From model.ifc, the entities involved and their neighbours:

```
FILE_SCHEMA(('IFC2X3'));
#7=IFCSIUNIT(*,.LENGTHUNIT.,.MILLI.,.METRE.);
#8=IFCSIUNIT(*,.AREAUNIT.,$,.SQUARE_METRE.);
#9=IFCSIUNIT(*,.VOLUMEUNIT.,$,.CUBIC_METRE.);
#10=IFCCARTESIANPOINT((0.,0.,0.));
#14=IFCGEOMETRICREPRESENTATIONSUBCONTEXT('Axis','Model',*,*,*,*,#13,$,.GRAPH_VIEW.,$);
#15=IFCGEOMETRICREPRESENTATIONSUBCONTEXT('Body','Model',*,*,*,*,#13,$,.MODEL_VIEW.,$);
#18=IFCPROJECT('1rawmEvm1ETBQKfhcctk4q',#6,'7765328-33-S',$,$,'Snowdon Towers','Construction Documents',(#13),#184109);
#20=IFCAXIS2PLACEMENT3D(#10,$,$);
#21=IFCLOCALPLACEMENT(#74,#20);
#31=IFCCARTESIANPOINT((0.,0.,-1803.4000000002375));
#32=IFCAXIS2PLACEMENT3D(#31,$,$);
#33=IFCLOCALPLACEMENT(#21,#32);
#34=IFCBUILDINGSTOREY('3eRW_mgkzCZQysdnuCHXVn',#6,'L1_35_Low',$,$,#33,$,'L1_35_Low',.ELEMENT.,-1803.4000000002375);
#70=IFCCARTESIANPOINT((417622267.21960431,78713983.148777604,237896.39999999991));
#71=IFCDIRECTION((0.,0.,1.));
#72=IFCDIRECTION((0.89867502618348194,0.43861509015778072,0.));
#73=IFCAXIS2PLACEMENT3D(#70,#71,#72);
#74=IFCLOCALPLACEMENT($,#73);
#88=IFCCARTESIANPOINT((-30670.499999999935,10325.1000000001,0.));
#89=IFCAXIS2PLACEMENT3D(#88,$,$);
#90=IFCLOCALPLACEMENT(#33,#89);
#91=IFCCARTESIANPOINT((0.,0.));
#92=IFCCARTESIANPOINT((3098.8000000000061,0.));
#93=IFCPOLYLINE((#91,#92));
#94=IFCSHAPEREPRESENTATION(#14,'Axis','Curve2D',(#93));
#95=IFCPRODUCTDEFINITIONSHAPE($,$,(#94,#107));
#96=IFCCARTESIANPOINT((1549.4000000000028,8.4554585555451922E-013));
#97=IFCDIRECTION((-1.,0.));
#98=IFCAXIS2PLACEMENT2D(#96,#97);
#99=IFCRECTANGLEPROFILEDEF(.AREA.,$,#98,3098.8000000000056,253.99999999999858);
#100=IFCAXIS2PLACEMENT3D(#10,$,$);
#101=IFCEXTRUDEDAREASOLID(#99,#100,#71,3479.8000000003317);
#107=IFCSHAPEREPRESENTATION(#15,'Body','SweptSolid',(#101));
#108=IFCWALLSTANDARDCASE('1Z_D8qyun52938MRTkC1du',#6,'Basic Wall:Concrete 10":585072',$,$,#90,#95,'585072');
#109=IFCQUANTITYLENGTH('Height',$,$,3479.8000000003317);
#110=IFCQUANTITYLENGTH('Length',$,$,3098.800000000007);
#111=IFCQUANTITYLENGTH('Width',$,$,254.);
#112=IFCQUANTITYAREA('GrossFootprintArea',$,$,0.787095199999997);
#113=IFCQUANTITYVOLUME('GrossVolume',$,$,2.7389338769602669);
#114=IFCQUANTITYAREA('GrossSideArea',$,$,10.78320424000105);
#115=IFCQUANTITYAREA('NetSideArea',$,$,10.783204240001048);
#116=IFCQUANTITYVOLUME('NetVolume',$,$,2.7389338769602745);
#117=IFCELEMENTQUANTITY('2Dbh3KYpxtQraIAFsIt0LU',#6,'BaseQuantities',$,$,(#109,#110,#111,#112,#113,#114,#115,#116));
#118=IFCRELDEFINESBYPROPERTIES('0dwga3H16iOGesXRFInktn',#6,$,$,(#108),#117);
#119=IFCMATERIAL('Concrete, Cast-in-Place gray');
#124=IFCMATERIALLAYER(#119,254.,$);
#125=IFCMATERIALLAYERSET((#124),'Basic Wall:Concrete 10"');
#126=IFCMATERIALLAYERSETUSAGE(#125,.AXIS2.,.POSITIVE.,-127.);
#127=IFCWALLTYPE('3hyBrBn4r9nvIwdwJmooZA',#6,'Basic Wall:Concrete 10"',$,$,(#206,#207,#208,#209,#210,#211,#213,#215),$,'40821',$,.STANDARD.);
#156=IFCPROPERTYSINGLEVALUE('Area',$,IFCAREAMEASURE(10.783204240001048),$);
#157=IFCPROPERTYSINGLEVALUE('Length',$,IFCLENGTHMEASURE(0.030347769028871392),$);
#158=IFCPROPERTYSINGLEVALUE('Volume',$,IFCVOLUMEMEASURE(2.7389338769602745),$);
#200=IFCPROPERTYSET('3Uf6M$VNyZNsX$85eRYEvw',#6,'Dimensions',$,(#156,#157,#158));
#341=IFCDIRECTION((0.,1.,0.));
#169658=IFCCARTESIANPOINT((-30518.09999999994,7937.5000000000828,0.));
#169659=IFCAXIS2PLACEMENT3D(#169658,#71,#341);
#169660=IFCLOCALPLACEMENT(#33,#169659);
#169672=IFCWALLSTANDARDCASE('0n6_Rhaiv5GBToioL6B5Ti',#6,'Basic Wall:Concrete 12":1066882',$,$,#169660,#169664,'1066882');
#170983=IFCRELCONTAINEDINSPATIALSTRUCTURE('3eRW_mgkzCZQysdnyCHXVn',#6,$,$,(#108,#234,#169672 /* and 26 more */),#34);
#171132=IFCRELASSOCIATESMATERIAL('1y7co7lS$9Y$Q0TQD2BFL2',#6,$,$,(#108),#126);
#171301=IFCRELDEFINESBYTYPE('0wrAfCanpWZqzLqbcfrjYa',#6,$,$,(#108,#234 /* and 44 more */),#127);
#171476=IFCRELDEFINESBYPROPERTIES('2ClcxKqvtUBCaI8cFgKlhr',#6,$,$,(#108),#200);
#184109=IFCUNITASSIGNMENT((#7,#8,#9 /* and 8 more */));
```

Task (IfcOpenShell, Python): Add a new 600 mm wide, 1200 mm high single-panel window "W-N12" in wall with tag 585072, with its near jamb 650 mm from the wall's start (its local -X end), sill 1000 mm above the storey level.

```python
import numpy as np
import ifcopenshell
import ifcopenshell.api.feature
import ifcopenshell.api.geometry
import ifcopenshell.api.pset
import ifcopenshell.api.root
import ifcopenshell.api.spatial
import ifcopenshell.api.type
import ifcopenshell.geom
import ifcopenshell.util.element
import ifcopenshell.util.placement
import ifcopenshell.util.representation
import ifcopenshell.util.shape
import ifcopenshell.util.unit

model = ifcopenshell.open("model.ifc")
unit_scale = ifcopenshell.util.unit.calculate_unit_scale(model)
area_scale = ifcopenshell.util.unit.calculate_unit_scale(model, "AREAUNIT")
volume_scale = ifcopenshell.util.unit.calculate_unit_scale(model, "VOLUMEUNIT")
settings = ifcopenshell.geom.settings()


def volume(element):
    """Net volume in cubic metres, openings subtracted."""
    shape = ifcopenshell.geom.create_shape(settings, element)
    return ifcopenshell.util.shape.get_volume(shape.geometry)


wall = model.by_guid("1Z_D8qyun52938MRTkC1du")
storey = ifcopenshell.util.element.get_container(wall, ifc_class="IfcBuildingStorey")
context = ifcopenshell.util.representation.get_context(model, "Model", "Body", "MODEL_VIEW")
before = volume(wall)

width, height, from_end, sill = 0.6, 1.2, 0.65, 1  # metres

# The wall runs along its own X axis, and the end named is its -X end.
wall_shape = ifcopenshell.geom.create_shape(settings, wall)
x, y, z = ifcopenshell.util.shape.get_vertices(wall_shape.geometry).T
start = x.min() + from_end
face, thickness = float(y.min()), float(y.max() - y.min())
wall_matrix = ifcopenshell.util.placement.get_local_placement(wall.ObjectPlacement)
level = ifcopenshell.util.placement.get_local_placement(storey.ObjectPlacement)[2, 3]


def in_wall(x, y):
    """Placement at x, y metres in the wall's axes, at sill height."""
    matrix = wall_matrix.copy()
    matrix[:, 3] = wall_matrix @ np.array([x / unit_scale, y / unit_scale, 0.0, 1.0])
    matrix[2, 3] = level + sill / unit_scale
    return matrix


# Opening: a box that overshoots both wall faces by 50 mm.
opening = ifcopenshell.api.root.create_entity(model, ifc_class="IfcOpeningElement")
box = ifcopenshell.api.geometry.add_wall_representation(
    model, context=context, length=width, height=height, thickness=thickness + 0.1
)
ifcopenshell.api.geometry.assign_representation(model, product=opening, representation=box)
ifcopenshell.api.geometry.edit_object_placement(model, product=opening, matrix=in_wall(start, face - 0.05), is_si=False)
ifcopenshell.api.feature.add_feature(model, feature=opening, element=wall)

window = ifcopenshell.api.root.create_entity(model, ifc_class="IfcWindow", name="W-N12")
window.OverallWidth, window.OverallHeight = width / unit_scale, height / unit_scale
body = ifcopenshell.api.geometry.add_window_representation(
    model,
    context=context,
    overall_width=window.OverallWidth,
    overall_height=window.OverallHeight,
    partition_type="SINGLE_PANEL",
)
ifcopenshell.api.geometry.assign_representation(model, product=window, representation=body)
ifcopenshell.api.spatial.assign_container(model, products=[window], relating_structure=storey)
fills = ifcopenshell.api.feature.add_filling(model, opening=opening, element=window)
fills.OwnerHistory = window.OwnerHistory  # required in IFC2X3

# IFC2X3 keeps the operation on the window style.
style = ifcopenshell.api.root.create_entity(model, ifc_class="IfcWindowStyle", name="W-N12")
style.OperationType, style.ConstructionType = "SINGLE_PANEL", "NOTDEFINED"
style.ParameterTakesPrecedence = style.Sizeable = False
ifcopenshell.api.type.assign_type(model, related_objects=[window], relating_type=style)

# Centre the window in the wall's thickness.
ifcopenshell.api.geometry.edit_object_placement(model, product=window, matrix=in_wall(start, face), is_si=False)
window_shape = ifcopenshell.geom.create_shape(settings, window)
depth = ifcopenshell.util.shape.get_vertices(window_shape.geometry)[:, 1]
offset = face + thickness / 2 - (depth.min() + depth.max()) / 2
ifcopenshell.api.geometry.edit_object_placement(model, product=window, matrix=in_wall(start, offset), is_si=False)

after = volume(wall)

# Update the wall's stored quantities.
qto = model.by_id(ifcopenshell.util.element.get_pset(wall, "BaseQuantities", should_inherit=False)["id"])
ifcopenshell.api.pset.edit_qto(model, qto=qto, properties={
    "NetSideArea": after / thickness / area_scale,
    "NetVolume": after / volume_scale,
})
pset = model.by_id(ifcopenshell.util.element.get_pset(wall, "Dimensions", should_inherit=False)["id"])
ifcopenshell.api.pset.edit_pset(model, pset=pset, properties={
    "Area": model.create_entity("IfcAreaMeasure", after / thickness / area_scale),
    "Volume": model.create_entity("IfcVolumeMeasure", after / volume_scale),
})

print(f"wall volume {before:.3f} -> {after:.3f} m3")

model.write("model_updated.ifc")
```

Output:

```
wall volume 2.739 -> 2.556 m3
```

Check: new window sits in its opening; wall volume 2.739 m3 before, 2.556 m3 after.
